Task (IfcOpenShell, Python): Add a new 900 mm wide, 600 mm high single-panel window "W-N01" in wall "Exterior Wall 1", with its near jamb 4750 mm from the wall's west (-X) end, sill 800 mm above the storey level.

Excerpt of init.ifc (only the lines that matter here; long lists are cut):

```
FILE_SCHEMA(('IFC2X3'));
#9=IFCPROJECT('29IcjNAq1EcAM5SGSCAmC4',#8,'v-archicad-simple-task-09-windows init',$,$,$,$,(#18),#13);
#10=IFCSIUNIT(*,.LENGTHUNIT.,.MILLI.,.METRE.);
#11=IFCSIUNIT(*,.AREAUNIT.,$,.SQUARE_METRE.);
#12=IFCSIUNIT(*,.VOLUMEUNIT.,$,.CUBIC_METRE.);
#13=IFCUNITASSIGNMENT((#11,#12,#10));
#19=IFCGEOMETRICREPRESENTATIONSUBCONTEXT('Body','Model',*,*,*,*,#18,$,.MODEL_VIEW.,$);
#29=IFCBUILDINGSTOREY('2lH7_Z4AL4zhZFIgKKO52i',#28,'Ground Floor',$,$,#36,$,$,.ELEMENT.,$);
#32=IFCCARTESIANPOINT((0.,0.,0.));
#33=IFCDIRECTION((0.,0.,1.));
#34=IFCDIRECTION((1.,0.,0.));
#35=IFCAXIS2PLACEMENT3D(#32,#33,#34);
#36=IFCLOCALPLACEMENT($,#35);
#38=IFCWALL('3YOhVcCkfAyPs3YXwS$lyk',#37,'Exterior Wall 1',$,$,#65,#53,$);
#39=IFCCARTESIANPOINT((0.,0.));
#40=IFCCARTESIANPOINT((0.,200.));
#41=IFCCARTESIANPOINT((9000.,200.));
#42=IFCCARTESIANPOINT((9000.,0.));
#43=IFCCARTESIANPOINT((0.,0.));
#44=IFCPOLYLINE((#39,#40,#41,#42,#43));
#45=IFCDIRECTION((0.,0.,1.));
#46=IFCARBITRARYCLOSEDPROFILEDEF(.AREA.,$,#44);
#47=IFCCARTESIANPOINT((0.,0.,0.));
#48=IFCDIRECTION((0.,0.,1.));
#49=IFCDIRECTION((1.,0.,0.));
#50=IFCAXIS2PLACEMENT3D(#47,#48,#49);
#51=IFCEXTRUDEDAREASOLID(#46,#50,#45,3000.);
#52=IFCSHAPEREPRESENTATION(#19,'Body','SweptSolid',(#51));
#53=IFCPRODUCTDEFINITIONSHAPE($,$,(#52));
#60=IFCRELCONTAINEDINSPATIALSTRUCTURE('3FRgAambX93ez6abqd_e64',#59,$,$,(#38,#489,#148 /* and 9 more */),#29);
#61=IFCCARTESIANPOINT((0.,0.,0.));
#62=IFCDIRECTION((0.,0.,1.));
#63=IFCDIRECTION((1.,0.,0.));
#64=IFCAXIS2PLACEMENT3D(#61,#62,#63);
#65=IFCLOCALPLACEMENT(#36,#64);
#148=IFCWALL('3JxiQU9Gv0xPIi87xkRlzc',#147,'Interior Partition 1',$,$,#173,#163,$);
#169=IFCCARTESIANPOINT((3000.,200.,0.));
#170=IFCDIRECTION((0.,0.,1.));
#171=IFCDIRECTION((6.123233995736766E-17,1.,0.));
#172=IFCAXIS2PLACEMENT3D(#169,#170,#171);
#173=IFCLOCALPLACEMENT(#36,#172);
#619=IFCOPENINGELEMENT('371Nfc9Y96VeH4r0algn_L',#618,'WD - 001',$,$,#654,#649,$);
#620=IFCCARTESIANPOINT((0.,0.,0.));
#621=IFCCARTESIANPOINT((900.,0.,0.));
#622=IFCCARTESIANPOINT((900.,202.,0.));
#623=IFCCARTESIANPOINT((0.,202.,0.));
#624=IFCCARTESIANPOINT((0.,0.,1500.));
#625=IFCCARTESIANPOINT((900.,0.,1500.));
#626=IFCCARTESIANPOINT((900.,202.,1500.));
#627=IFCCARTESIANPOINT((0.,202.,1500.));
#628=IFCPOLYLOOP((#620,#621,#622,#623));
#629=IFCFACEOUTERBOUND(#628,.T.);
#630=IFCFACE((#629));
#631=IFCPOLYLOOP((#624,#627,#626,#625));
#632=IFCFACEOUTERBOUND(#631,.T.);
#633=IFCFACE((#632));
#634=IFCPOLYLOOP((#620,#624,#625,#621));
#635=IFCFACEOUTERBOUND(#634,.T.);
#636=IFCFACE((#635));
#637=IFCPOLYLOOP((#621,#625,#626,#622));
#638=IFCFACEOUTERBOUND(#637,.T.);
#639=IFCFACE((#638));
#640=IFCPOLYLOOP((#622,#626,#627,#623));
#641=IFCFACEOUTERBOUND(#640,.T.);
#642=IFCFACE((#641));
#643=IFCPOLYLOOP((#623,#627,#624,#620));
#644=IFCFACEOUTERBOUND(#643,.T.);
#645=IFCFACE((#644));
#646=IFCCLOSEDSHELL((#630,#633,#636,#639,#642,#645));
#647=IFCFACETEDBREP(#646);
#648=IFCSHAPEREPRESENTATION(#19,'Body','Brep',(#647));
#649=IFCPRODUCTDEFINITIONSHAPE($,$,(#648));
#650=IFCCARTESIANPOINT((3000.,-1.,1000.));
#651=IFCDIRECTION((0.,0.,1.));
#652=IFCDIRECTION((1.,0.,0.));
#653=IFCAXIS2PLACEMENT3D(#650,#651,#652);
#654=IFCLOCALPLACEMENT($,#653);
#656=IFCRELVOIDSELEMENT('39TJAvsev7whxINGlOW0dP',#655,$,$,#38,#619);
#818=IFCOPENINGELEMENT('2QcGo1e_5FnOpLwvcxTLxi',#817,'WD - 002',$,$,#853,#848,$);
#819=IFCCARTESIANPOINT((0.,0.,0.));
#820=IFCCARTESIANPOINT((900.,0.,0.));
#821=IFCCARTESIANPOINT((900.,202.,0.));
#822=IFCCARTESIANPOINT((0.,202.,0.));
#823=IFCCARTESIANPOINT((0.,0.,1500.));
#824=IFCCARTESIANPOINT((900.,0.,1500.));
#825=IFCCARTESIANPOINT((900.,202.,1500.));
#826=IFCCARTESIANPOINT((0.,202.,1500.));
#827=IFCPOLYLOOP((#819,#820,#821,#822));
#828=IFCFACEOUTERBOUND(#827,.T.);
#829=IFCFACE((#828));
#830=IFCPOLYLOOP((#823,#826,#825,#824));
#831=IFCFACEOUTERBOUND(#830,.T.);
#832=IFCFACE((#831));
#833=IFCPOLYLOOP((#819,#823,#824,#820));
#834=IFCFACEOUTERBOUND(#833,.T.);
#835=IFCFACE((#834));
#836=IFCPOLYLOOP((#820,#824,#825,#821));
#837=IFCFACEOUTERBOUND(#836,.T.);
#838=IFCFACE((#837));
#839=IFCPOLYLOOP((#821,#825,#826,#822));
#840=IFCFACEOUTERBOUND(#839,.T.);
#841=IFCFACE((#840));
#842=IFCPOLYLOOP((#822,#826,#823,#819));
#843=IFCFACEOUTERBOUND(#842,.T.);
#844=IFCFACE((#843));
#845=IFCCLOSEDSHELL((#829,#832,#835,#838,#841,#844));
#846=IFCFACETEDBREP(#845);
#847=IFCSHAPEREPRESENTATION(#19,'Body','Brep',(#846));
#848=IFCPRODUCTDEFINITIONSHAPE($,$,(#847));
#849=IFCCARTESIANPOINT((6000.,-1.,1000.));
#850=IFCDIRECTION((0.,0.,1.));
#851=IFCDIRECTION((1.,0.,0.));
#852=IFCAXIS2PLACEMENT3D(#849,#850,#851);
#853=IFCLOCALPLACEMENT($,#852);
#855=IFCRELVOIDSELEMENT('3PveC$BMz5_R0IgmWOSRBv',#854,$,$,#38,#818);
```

```python
import numpy as np
import ifcopenshell
import ifcopenshell.api.feature
import ifcopenshell.api.geometry
import ifcopenshell.api.root
import ifcopenshell.api.spatial
import ifcopenshell.api.type
import ifcopenshell.geom
import ifcopenshell.util.element
import ifcopenshell.util.placement
import ifcopenshell.util.representation
import ifcopenshell.util.shape
import ifcopenshell.util.unit

model = ifcopenshell.open("init.ifc")
unit_scale = ifcopenshell.util.unit.calculate_unit_scale(model)
settings = ifcopenshell.geom.settings()


def volume(element):
    """Net volume in cubic metres, openings subtracted."""
    shape = ifcopenshell.geom.create_shape(settings, element)
    return ifcopenshell.util.shape.get_volume(shape.geometry)


wall = model.by_guid("3YOhVcCkfAyPs3YXwS$lyk")
storey = ifcopenshell.util.element.get_container(wall, ifc_class="IfcBuildingStorey")
context = ifcopenshell.util.representation.get_context(model, "Model", "Body", "MODEL_VIEW")
before = volume(wall)

width, height, from_end, sill = 0.9, 0.6, 4.75, 0.8  # metres

# The wall runs along its own X axis, and the end named is its -X end.
wall_shape = ifcopenshell.geom.create_shape(settings, wall)
x, y, z = ifcopenshell.util.shape.get_vertices(wall_shape.geometry).T
start = x.min() + from_end
face, thickness = float(y.min()), float(y.max() - y.min())
wall_matrix = ifcopenshell.util.placement.get_local_placement(wall.ObjectPlacement)
level = ifcopenshell.util.placement.get_local_placement(storey.ObjectPlacement)[2, 3]


def in_wall(x, y):
    """Placement at x, y metres in the wall's axes, at sill height."""
    matrix = wall_matrix.copy()
    matrix[:, 3] = wall_matrix @ np.array([x / unit_scale, y / unit_scale, 0.0, 1.0])
    matrix[2, 3] = level + sill / unit_scale
    return matrix


# Opening: a box that overshoots both wall faces by 50 mm.
opening = ifcopenshell.api.root.create_entity(model, ifc_class="IfcOpeningElement")
box = ifcopenshell.api.geometry.add_wall_representation(
    model, context=context, length=width, height=height, thickness=thickness + 0.1
)
ifcopenshell.api.geometry.assign_representation(model, product=opening, representation=box)
ifcopenshell.api.geometry.edit_object_placement(model, product=opening, matrix=in_wall(start, face - 0.05), is_si=False)
ifcopenshell.api.feature.add_feature(model, feature=opening, element=wall)

window = ifcopenshell.api.root.create_entity(model, ifc_class="IfcWindow", name="W-N01")
window.OverallWidth, window.OverallHeight = width / unit_scale, height / unit_scale
body = ifcopenshell.api.geometry.add_window_representation(
    model,
    context=context,
    overall_width=window.OverallWidth,
    overall_height=window.OverallHeight,
    partition_type="SINGLE_PANEL",
)
ifcopenshell.api.geometry.assign_representation(model, product=window, representation=body)
ifcopenshell.api.spatial.assign_container(model, products=[window], relating_structure=storey)
fills = ifcopenshell.api.feature.add_filling(model, opening=opening, element=window)
fills.OwnerHistory = window.OwnerHistory  # required in IFC2X3

# IFC2X3 keeps the operation on the window style.
style = ifcopenshell.api.root.create_entity(model, ifc_class="IfcWindowStyle", name="W-N01")
style.OperationType, style.ConstructionType = "SINGLE_PANEL", "NOTDEFINED"
style.ParameterTakesPrecedence = style.Sizeable = False
ifcopenshell.api.type.assign_type(model, related_objects=[window], relating_type=style)

# Centre the window in the wall's thickness.
ifcopenshell.api.geometry.edit_object_placement(model, product=window, matrix=in_wall(start, face), is_si=False)
window_shape = ifcopenshell.geom.create_shape(settings, window)
depth = ifcopenshell.util.shape.get_vertices(window_shape.geometry)[:, 1]
offset = face + thickness / 2 - (depth.min() + depth.max()) / 2
ifcopenshell.api.geometry.edit_object_placement(model, product=window, matrix=in_wall(start, offset), is_si=False)

after = volume(wall)

print(f"wall volume {before:.3f} -> {after:.3f} m3")

model.write("init_rev.ifc")
```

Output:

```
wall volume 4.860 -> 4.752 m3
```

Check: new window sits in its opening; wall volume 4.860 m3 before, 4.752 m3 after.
